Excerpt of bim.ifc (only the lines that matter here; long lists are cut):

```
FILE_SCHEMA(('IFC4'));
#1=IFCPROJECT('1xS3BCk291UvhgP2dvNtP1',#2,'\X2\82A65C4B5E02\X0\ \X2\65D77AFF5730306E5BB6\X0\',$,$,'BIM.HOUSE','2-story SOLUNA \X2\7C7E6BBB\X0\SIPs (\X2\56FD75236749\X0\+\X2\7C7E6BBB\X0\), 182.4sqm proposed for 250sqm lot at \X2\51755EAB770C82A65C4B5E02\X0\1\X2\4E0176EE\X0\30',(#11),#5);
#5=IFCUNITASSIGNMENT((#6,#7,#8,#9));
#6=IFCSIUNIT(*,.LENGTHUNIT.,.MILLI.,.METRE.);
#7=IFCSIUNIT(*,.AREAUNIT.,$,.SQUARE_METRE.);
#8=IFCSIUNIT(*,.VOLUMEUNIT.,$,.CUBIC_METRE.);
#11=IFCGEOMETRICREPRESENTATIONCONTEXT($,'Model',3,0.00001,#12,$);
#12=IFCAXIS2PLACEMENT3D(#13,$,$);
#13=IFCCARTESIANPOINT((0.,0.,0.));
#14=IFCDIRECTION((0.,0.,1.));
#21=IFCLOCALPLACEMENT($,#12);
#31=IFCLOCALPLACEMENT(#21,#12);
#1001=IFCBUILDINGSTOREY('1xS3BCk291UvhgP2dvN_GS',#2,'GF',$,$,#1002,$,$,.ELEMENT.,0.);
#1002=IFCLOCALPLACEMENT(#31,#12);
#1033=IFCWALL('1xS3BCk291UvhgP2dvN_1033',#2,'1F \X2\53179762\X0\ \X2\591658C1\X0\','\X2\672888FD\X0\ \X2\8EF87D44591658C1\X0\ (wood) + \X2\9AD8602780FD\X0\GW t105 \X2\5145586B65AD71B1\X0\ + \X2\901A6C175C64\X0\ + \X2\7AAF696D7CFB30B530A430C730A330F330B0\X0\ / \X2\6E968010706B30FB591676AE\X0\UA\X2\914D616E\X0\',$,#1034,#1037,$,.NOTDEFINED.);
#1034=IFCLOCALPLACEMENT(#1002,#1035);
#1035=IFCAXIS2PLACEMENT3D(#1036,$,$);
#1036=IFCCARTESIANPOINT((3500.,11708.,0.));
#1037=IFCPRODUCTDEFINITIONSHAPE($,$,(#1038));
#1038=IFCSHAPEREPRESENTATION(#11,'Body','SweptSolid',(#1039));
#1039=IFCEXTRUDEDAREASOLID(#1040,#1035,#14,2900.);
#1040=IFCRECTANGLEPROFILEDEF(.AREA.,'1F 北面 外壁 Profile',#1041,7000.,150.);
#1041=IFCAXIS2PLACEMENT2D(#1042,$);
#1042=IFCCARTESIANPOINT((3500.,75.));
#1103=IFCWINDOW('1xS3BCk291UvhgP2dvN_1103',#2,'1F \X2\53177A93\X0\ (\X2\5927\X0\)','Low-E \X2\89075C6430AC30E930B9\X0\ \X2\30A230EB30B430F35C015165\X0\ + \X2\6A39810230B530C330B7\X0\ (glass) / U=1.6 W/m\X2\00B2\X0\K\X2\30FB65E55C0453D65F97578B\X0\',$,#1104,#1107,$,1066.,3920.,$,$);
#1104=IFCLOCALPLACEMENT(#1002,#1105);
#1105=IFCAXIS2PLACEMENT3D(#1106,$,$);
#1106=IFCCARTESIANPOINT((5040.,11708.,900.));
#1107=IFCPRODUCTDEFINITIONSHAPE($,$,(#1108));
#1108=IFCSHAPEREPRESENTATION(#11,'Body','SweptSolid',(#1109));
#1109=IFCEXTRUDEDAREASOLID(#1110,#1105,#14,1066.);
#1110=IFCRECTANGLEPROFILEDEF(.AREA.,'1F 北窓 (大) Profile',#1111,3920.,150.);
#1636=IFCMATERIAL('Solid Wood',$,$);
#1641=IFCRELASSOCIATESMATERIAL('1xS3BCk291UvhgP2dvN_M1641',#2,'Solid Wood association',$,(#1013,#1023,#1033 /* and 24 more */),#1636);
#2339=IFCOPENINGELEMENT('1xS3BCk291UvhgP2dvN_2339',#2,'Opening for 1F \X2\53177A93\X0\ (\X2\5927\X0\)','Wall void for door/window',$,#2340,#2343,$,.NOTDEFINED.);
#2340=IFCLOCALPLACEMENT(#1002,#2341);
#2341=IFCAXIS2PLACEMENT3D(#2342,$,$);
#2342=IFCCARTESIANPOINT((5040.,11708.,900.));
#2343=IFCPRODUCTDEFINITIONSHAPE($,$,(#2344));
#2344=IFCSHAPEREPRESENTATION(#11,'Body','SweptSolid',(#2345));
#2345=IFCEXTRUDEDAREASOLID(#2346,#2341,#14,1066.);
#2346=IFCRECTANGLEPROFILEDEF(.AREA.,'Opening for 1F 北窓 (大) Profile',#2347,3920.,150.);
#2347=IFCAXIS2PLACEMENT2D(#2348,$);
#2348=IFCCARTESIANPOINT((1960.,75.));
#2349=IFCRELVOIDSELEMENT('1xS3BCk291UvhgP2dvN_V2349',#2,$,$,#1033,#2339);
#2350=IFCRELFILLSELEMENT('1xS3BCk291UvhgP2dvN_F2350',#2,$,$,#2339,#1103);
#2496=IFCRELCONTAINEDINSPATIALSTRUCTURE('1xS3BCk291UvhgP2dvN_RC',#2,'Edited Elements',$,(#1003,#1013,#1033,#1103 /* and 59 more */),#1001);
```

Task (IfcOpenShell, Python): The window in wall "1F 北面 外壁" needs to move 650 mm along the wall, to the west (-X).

```python
import ifcopenshell
import ifcopenshell.api.geometry
import ifcopenshell.util.placement
import ifcopenshell.util.unit

model = ifcopenshell.open("bim.ifc")
unit_scale = ifcopenshell.util.unit.calculate_unit_scale(model)

window = model.by_id(1103)
opening = window.FillsVoids[0].RelatingOpeningElement
wall = opening.VoidsElements[0].RelatingBuildingElement

wall_matrix = ifcopenshell.util.placement.get_local_placement(wall.ObjectPlacement)
shift = wall_matrix[:3, 0] * -0.65 / unit_scale
before = ifcopenshell.util.placement.get_local_placement(window.ObjectPlacement)[:3, 3].copy()

# The window is not placed relative to its opening, so move both.
for product in (opening, window):
    matrix = ifcopenshell.util.placement.get_local_placement(product.ObjectPlacement)
    matrix[:3, 3] += shift
    ifcopenshell.api.geometry.edit_object_placement(model, product=product, matrix=matrix, is_si=False)

after = ifcopenshell.util.placement.get_local_placement(window.ObjectPlacement)[:3, 3]
print("window moved by", (after - before).round(3) + 0.0)

model.write("bim_edited.ifc")
```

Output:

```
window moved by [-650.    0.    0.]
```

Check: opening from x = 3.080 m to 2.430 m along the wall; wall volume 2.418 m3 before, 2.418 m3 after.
